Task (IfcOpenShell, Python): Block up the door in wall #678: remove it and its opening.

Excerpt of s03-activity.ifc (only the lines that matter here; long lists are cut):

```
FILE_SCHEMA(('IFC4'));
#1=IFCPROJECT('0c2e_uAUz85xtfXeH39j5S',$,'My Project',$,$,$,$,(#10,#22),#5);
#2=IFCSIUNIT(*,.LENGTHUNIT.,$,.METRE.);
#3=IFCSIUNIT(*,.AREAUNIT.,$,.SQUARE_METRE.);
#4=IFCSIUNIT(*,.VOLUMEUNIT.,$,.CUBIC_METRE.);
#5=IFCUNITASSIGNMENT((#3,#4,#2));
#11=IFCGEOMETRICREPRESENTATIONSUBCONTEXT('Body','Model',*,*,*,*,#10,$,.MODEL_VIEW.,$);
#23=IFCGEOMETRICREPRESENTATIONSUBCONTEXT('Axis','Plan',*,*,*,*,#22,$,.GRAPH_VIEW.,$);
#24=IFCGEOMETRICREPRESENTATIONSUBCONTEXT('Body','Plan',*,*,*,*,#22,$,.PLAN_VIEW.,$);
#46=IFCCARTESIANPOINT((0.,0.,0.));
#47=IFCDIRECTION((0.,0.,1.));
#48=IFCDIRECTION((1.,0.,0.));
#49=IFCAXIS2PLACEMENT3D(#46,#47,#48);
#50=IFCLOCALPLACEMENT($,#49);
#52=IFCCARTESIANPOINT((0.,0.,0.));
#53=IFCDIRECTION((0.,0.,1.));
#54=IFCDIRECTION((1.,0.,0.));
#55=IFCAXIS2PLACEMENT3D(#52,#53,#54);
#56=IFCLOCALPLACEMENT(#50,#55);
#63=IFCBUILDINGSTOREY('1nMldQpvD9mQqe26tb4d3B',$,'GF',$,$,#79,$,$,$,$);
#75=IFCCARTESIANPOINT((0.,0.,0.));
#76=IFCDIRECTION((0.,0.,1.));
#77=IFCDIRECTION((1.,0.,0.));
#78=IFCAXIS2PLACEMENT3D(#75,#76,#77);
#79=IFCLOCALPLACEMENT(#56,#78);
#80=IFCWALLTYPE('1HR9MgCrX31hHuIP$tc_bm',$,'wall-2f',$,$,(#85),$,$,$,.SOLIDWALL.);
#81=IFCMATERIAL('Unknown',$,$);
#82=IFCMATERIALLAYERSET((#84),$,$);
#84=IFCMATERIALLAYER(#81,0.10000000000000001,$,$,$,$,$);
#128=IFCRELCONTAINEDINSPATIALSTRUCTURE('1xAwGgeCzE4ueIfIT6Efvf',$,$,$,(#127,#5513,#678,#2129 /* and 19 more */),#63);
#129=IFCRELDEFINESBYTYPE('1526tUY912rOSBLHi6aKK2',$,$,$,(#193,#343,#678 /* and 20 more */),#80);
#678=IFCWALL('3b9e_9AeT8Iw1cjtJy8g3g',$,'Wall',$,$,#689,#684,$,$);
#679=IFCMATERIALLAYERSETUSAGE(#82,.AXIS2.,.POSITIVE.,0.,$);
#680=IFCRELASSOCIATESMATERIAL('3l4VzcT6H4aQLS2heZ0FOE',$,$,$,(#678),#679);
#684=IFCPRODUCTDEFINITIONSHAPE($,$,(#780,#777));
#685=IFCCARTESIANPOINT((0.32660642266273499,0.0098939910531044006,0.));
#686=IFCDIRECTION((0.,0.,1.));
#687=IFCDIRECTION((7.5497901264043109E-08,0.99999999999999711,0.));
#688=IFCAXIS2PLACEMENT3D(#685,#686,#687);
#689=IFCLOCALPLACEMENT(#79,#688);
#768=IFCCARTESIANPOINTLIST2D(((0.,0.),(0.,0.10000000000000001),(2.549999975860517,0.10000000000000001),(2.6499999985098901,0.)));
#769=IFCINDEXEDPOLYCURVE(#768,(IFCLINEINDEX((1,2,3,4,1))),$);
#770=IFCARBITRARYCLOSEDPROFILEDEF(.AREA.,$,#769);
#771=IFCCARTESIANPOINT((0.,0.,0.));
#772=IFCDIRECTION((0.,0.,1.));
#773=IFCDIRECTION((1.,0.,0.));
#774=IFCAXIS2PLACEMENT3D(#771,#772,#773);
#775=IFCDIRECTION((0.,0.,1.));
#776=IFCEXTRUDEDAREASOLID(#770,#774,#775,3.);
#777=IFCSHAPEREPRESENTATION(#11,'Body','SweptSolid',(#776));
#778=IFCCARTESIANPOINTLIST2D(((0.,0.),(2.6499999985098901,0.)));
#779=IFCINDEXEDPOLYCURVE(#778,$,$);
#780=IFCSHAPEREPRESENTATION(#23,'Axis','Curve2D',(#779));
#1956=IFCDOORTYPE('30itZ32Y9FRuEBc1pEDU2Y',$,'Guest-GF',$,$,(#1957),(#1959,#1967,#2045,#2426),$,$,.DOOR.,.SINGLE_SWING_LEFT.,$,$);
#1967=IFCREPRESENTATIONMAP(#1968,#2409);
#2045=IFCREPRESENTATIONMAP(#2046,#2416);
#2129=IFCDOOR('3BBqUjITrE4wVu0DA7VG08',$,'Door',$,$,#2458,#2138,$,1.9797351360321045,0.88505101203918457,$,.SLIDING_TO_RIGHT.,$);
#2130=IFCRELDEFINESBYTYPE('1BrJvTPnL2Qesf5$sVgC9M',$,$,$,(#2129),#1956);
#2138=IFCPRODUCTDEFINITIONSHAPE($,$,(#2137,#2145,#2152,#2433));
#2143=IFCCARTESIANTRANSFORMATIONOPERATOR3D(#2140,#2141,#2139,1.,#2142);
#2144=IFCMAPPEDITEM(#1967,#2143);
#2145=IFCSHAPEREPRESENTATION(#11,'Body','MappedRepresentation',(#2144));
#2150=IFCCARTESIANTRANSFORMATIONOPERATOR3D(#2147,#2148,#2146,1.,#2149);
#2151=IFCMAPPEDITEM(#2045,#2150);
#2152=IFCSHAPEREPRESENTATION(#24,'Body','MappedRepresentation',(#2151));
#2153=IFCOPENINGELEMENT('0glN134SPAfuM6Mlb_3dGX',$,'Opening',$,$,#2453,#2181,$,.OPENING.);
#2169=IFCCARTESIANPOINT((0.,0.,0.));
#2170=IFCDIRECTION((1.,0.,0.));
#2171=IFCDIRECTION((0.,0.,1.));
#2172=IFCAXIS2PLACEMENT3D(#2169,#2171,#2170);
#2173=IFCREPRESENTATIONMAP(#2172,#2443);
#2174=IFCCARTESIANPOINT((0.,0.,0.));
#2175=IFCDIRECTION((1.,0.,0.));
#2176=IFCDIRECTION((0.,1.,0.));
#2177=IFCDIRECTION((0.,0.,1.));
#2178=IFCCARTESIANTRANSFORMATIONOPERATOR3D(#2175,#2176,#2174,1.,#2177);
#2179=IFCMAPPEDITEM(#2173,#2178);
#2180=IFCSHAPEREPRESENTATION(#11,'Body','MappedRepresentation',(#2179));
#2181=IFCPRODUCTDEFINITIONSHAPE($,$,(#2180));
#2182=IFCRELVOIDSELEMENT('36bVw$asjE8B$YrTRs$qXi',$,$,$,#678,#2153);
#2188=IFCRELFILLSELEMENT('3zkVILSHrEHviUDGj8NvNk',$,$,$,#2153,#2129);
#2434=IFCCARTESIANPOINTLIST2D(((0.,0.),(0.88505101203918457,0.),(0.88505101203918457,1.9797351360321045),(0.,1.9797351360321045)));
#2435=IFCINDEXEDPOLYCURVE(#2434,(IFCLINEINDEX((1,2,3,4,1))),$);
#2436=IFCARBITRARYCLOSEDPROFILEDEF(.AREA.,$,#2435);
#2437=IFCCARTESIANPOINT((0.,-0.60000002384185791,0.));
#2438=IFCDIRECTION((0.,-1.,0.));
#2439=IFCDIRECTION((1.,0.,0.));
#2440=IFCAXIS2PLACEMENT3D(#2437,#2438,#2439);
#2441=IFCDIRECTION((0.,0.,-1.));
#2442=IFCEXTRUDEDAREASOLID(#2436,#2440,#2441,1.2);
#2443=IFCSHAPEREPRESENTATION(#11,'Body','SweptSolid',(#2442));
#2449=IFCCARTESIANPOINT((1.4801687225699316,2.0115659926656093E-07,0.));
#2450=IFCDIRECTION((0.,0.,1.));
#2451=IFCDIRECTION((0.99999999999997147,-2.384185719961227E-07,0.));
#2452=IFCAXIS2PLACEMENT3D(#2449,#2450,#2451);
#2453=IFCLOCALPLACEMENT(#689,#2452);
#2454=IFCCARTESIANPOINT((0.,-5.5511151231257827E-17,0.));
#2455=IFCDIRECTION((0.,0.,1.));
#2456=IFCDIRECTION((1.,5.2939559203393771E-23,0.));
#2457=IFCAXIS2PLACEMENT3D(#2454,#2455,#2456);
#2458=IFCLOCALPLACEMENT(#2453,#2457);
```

```python
import ifcopenshell
import ifcopenshell.api.feature
import ifcopenshell.api.root
import ifcopenshell.geom
import ifcopenshell.util.shape

model = ifcopenshell.open("s03-activity.ifc")
settings = ifcopenshell.geom.settings()


def volume(element):
    """Net volume in cubic metres, openings subtracted."""
    shape = ifcopenshell.geom.create_shape(settings, element)
    return ifcopenshell.util.shape.get_volume(shape.geometry)


door = model.by_guid("3BBqUjITrE4wVu0DA7VG08")
opening = door.FillsVoids[0].RelatingOpeningElement
wall = opening.VoidsElements[0].RelatingBuildingElement
before = volume(wall)

ifcopenshell.api.root.remove_product(model, product=door)
ifcopenshell.api.feature.remove_feature(model, feature=opening)

after = volume(wall)

print(f"wall volume {before:.3f} -> {after:.3f} m3")

model.write("s03-activity_v2.ifc")
```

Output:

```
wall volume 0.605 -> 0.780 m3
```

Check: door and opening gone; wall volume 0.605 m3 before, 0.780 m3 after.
